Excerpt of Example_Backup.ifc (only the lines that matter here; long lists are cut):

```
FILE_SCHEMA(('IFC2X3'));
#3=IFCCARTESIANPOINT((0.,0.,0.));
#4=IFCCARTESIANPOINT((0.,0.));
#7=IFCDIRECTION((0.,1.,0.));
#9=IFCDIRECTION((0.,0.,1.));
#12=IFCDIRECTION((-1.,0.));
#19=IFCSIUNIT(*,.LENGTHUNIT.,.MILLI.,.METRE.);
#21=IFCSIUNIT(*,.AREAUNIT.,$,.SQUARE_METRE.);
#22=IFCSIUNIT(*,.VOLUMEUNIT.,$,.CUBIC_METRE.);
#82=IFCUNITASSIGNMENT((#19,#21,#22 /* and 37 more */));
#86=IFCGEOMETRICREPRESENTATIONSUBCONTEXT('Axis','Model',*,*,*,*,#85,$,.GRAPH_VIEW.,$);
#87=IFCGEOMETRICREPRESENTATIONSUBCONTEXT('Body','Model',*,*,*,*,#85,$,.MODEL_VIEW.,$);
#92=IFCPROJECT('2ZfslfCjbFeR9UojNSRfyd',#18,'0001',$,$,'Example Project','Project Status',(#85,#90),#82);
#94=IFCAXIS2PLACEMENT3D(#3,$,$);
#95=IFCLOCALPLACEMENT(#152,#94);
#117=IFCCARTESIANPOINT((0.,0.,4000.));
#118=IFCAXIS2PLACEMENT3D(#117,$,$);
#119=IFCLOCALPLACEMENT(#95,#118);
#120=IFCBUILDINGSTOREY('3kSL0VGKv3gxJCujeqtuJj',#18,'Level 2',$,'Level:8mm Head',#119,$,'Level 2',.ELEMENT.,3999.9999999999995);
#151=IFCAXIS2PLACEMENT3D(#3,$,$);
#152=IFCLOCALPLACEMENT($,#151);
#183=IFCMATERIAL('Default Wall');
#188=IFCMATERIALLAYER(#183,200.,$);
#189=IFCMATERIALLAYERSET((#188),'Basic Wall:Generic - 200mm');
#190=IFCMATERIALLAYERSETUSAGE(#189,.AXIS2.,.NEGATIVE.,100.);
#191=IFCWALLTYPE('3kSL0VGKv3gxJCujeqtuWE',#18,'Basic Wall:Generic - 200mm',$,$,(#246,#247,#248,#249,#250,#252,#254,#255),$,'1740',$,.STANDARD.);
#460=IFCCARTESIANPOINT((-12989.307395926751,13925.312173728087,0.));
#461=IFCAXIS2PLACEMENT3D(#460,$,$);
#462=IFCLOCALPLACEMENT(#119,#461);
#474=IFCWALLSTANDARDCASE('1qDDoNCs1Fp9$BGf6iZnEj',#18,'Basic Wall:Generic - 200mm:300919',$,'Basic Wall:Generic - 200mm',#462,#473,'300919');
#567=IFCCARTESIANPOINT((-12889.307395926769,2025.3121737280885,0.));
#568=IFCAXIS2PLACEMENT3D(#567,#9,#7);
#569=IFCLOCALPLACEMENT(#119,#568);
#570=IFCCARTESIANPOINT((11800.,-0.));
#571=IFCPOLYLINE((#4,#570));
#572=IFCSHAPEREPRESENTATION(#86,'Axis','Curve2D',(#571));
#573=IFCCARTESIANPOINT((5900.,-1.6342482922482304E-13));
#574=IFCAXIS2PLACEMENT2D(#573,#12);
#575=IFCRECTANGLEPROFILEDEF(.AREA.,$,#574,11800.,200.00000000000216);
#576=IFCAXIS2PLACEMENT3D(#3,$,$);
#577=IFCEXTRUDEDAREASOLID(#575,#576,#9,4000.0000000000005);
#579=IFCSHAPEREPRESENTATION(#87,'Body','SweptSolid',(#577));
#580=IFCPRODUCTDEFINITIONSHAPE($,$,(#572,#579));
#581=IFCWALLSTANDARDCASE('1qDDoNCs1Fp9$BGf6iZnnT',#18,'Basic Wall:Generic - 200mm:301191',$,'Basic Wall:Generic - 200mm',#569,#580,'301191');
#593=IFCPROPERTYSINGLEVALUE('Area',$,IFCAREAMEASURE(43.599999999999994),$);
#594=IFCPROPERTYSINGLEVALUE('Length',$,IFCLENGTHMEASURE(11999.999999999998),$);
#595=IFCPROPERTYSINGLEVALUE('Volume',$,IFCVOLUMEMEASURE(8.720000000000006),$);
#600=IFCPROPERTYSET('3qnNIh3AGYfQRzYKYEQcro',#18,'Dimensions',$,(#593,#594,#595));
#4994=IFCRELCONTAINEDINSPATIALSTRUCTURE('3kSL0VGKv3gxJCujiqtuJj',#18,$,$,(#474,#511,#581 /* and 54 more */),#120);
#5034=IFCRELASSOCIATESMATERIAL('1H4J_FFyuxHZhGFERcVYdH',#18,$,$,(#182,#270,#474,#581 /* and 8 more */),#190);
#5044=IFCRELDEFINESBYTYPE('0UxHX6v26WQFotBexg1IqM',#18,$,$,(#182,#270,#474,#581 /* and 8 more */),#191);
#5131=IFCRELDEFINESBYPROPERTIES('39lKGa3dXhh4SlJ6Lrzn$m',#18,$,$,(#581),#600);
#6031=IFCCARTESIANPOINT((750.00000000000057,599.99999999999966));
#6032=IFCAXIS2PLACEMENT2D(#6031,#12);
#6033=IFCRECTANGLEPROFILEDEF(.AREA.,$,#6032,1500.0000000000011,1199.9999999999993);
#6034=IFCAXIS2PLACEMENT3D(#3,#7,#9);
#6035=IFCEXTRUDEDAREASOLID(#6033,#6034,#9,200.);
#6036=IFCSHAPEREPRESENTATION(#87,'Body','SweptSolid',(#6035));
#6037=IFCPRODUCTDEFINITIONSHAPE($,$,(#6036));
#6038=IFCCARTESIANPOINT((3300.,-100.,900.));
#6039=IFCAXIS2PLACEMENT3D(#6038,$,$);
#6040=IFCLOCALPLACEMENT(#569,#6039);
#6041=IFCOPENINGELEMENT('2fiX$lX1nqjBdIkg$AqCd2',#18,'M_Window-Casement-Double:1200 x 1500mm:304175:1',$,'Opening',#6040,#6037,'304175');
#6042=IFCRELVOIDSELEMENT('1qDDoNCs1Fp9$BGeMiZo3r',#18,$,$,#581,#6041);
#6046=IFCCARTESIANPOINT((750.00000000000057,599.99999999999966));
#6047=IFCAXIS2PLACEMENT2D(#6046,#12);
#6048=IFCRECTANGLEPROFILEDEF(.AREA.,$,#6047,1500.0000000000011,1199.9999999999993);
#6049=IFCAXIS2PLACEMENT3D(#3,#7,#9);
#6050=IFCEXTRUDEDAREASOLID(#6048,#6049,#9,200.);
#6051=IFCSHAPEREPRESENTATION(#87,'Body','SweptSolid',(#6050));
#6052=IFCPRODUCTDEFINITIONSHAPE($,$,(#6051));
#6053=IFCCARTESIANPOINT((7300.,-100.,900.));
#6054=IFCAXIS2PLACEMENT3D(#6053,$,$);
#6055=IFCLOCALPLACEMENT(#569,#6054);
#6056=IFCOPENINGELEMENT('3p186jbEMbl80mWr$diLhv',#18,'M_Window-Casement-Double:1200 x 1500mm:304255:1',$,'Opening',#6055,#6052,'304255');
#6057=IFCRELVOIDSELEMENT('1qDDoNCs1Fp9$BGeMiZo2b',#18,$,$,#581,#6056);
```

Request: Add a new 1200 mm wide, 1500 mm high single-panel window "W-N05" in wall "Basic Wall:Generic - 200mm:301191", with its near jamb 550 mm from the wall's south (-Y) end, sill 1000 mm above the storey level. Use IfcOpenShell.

```python
import numpy as np
import ifcopenshell
import ifcopenshell.api.feature
import ifcopenshell.api.geometry
import ifcopenshell.api.pset
import ifcopenshell.api.root
import ifcopenshell.api.spatial
import ifcopenshell.api.type
import ifcopenshell.geom
import ifcopenshell.util.element
import ifcopenshell.util.placement
import ifcopenshell.util.representation
import ifcopenshell.util.shape
import ifcopenshell.util.unit

model = ifcopenshell.open("Example_Backup.ifc")
unit_scale = ifcopenshell.util.unit.calculate_unit_scale(model)
area_scale = ifcopenshell.util.unit.calculate_unit_scale(model, "AREAUNIT")
volume_scale = ifcopenshell.util.unit.calculate_unit_scale(model, "VOLUMEUNIT")
settings = ifcopenshell.geom.settings()


def volume(element):
    """Net volume in cubic metres, openings subtracted."""
    shape = ifcopenshell.geom.create_shape(settings, element)
    return ifcopenshell.util.shape.get_volume(shape.geometry)


wall = model.by_guid("1qDDoNCs1Fp9$BGf6iZnnT")
storey = ifcopenshell.util.element.get_container(wall, ifc_class="IfcBuildingStorey")
context = ifcopenshell.util.representation.get_context(model, "Model", "Body", "MODEL_VIEW")
before = volume(wall)

width, height, from_end, sill = 1.2, 1.5, 0.55, 1  # metres

# The wall runs along its own X axis, and the end named is its -X end.
wall_shape = ifcopenshell.geom.create_shape(settings, wall)
x, y, z = ifcopenshell.util.shape.get_vertices(wall_shape.geometry).T
start = x.min() + from_end
face, thickness = float(y.min()), float(y.max() - y.min())
wall_matrix = ifcopenshell.util.placement.get_local_placement(wall.ObjectPlacement)
level = ifcopenshell.util.placement.get_local_placement(storey.ObjectPlacement)[2, 3]


def in_wall(x, y):
    """Placement at x, y metres in the wall's axes, at sill height."""
    matrix = wall_matrix.copy()
    matrix[:, 3] = wall_matrix @ np.array([x / unit_scale, y / unit_scale, 0.0, 1.0])
    matrix[2, 3] = level + sill / unit_scale
    return matrix


# Opening: a box that overshoots both wall faces by 50 mm.
opening = ifcopenshell.api.root.create_entity(model, ifc_class="IfcOpeningElement")
box = ifcopenshell.api.geometry.add_wall_representation(
    model, context=context, length=width, height=height, thickness=thickness + 0.1
)
ifcopenshell.api.geometry.assign_representation(model, product=opening, representation=box)
ifcopenshell.api.geometry.edit_object_placement(model, product=opening, matrix=in_wall(start, face - 0.05), is_si=False)
ifcopenshell.api.feature.add_feature(model, feature=opening, element=wall)

window = ifcopenshell.api.root.create_entity(model, ifc_class="IfcWindow", name="W-N05")
window.OverallWidth, window.OverallHeight = width / unit_scale, height / unit_scale
body = ifcopenshell.api.geometry.add_window_representation(
    model,
    context=context,
    overall_width=window.OverallWidth,
    overall_height=window.OverallHeight,
    partition_type="SINGLE_PANEL",
)
ifcopenshell.api.geometry.assign_representation(model, product=window, representation=body)
ifcopenshell.api.spatial.assign_container(model, products=[window], relating_structure=storey)
fills = ifcopenshell.api.feature.add_filling(model, opening=opening, element=window)
fills.OwnerHistory = window.OwnerHistory  # required in IFC2X3

# IFC2X3 keeps the operation on the window style.
style = ifcopenshell.api.root.create_entity(model, ifc_class="IfcWindowStyle", name="W-N05")
style.OperationType, style.ConstructionType = "SINGLE_PANEL", "NOTDEFINED"
style.ParameterTakesPrecedence = style.Sizeable = False
ifcopenshell.api.type.assign_type(model, related_objects=[window], relating_type=style)

# Centre the window in the wall's thickness.
ifcopenshell.api.geometry.edit_object_placement(model, product=window, matrix=in_wall(start, face), is_si=False)
window_shape = ifcopenshell.geom.create_shape(settings, window)
depth = ifcopenshell.util.shape.get_vertices(window_shape.geometry)[:, 1]
offset = face + thickness / 2 - (depth.min() + depth.max()) / 2
ifcopenshell.api.geometry.edit_object_placement(model, product=window, matrix=in_wall(start, offset), is_si=False)

after = volume(wall)

# Update the wall's stored quantities.
pset = model.by_id(ifcopenshell.util.element.get_pset(wall, "Dimensions", should_inherit=False)["id"])
ifcopenshell.api.pset.edit_pset(model, pset=pset, properties={
    "Area": model.create_entity("IfcAreaMeasure", after / thickness / area_scale),
    "Volume": model.create_entity("IfcVolumeMeasure", after / volume_scale),
})

print(f"wall volume {before:.3f} -> {after:.3f} m3")

model.write("Example_Backup-out.ifc")
```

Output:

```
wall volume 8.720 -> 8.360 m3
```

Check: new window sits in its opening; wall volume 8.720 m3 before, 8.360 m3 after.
